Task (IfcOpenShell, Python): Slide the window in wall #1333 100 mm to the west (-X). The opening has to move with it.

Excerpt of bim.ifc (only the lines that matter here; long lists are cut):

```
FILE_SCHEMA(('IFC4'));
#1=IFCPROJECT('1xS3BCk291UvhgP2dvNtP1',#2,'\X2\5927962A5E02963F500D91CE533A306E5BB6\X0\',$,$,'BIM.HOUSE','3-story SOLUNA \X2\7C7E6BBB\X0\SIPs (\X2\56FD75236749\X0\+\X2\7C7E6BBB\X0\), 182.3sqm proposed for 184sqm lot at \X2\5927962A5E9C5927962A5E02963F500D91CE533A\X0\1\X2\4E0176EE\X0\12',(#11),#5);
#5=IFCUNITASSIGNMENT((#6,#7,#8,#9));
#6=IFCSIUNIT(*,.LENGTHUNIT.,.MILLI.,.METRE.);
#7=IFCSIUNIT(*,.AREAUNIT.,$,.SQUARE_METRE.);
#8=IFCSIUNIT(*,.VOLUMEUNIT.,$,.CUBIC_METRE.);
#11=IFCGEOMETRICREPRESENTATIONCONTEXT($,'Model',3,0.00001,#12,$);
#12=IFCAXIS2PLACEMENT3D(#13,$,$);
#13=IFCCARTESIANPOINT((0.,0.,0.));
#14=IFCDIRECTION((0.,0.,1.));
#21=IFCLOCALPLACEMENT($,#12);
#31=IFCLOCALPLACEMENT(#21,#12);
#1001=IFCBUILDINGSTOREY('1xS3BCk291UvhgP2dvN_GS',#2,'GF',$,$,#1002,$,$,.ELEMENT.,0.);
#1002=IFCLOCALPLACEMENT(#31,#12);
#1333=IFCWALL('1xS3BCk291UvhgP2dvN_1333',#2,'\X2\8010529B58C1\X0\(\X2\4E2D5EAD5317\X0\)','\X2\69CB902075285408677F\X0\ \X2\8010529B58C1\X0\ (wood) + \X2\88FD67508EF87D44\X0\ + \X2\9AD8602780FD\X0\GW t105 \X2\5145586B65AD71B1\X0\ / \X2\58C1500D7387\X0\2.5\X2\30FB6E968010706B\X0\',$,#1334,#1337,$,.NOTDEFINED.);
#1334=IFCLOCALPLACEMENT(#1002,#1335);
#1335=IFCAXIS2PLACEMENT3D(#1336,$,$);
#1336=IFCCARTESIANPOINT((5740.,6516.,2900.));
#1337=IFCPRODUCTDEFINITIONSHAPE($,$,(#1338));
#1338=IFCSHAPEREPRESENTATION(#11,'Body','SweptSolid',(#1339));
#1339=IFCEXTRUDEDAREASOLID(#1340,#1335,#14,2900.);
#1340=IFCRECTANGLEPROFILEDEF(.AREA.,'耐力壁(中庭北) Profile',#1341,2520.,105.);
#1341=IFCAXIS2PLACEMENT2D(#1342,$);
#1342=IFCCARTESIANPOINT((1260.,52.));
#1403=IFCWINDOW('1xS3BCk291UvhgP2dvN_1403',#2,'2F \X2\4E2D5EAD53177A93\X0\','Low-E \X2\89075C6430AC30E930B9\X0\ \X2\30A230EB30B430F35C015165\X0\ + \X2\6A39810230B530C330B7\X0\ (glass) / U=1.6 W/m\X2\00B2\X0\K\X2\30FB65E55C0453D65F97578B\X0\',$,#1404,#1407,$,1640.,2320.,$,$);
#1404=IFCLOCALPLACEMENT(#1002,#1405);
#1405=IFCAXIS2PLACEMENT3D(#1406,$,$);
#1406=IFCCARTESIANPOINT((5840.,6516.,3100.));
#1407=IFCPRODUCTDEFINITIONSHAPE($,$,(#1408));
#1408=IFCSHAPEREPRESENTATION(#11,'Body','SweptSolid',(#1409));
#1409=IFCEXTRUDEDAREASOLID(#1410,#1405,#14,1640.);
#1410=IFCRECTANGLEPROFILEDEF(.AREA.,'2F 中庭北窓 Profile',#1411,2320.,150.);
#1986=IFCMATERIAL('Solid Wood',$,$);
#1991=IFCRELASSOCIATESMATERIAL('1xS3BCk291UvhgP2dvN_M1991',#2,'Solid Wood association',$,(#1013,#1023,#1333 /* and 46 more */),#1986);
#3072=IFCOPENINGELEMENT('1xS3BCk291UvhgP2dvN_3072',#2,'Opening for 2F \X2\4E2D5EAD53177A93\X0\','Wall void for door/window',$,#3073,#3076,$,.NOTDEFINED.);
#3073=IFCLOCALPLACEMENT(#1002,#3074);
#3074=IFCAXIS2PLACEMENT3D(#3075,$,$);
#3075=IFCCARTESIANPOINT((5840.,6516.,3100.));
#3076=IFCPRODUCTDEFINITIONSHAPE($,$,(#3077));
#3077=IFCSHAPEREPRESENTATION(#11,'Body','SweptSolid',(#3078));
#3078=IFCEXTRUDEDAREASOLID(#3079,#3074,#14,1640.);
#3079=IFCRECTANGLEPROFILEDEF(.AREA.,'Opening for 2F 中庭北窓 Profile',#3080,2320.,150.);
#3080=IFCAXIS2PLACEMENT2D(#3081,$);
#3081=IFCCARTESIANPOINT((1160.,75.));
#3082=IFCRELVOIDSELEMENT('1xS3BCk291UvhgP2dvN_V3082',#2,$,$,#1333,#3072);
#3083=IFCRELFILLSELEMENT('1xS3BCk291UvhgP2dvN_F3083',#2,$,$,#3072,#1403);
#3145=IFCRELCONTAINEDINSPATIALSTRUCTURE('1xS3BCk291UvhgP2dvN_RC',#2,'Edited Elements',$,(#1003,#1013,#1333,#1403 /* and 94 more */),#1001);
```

```python
import ifcopenshell
import ifcopenshell.api.geometry
import ifcopenshell.util.placement

model = ifcopenshell.open("bim.ifc")

window = model.by_guid("1xS3BCk291UvhgP2dvN_1403")
opening = window.FillsVoids[0].RelatingOpeningElement
wall = opening.VoidsElements[0].RelatingBuildingElement

wall_matrix = ifcopenshell.util.placement.get_local_placement(wall.ObjectPlacement)
shift = wall_matrix[:3, 0] * -100.0
before = ifcopenshell.util.placement.get_local_placement(window.ObjectPlacement)[:3, 3].copy()

# The window is not placed relative to its opening, so move both.
for product in (opening, window):
    matrix = ifcopenshell.util.placement.get_local_placement(product.ObjectPlacement)
    matrix[:3, 3] += shift
    ifcopenshell.api.geometry.edit_object_placement(model, product=product, matrix=matrix, is_si=False)

after = ifcopenshell.util.placement.get_local_placement(window.ObjectPlacement)[:3, 3]
print("window moved by", (after - before).round(3) + 0.0)

model.write("bim-out.ifc")
```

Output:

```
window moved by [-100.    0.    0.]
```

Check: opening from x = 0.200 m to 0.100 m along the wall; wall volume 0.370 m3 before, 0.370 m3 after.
